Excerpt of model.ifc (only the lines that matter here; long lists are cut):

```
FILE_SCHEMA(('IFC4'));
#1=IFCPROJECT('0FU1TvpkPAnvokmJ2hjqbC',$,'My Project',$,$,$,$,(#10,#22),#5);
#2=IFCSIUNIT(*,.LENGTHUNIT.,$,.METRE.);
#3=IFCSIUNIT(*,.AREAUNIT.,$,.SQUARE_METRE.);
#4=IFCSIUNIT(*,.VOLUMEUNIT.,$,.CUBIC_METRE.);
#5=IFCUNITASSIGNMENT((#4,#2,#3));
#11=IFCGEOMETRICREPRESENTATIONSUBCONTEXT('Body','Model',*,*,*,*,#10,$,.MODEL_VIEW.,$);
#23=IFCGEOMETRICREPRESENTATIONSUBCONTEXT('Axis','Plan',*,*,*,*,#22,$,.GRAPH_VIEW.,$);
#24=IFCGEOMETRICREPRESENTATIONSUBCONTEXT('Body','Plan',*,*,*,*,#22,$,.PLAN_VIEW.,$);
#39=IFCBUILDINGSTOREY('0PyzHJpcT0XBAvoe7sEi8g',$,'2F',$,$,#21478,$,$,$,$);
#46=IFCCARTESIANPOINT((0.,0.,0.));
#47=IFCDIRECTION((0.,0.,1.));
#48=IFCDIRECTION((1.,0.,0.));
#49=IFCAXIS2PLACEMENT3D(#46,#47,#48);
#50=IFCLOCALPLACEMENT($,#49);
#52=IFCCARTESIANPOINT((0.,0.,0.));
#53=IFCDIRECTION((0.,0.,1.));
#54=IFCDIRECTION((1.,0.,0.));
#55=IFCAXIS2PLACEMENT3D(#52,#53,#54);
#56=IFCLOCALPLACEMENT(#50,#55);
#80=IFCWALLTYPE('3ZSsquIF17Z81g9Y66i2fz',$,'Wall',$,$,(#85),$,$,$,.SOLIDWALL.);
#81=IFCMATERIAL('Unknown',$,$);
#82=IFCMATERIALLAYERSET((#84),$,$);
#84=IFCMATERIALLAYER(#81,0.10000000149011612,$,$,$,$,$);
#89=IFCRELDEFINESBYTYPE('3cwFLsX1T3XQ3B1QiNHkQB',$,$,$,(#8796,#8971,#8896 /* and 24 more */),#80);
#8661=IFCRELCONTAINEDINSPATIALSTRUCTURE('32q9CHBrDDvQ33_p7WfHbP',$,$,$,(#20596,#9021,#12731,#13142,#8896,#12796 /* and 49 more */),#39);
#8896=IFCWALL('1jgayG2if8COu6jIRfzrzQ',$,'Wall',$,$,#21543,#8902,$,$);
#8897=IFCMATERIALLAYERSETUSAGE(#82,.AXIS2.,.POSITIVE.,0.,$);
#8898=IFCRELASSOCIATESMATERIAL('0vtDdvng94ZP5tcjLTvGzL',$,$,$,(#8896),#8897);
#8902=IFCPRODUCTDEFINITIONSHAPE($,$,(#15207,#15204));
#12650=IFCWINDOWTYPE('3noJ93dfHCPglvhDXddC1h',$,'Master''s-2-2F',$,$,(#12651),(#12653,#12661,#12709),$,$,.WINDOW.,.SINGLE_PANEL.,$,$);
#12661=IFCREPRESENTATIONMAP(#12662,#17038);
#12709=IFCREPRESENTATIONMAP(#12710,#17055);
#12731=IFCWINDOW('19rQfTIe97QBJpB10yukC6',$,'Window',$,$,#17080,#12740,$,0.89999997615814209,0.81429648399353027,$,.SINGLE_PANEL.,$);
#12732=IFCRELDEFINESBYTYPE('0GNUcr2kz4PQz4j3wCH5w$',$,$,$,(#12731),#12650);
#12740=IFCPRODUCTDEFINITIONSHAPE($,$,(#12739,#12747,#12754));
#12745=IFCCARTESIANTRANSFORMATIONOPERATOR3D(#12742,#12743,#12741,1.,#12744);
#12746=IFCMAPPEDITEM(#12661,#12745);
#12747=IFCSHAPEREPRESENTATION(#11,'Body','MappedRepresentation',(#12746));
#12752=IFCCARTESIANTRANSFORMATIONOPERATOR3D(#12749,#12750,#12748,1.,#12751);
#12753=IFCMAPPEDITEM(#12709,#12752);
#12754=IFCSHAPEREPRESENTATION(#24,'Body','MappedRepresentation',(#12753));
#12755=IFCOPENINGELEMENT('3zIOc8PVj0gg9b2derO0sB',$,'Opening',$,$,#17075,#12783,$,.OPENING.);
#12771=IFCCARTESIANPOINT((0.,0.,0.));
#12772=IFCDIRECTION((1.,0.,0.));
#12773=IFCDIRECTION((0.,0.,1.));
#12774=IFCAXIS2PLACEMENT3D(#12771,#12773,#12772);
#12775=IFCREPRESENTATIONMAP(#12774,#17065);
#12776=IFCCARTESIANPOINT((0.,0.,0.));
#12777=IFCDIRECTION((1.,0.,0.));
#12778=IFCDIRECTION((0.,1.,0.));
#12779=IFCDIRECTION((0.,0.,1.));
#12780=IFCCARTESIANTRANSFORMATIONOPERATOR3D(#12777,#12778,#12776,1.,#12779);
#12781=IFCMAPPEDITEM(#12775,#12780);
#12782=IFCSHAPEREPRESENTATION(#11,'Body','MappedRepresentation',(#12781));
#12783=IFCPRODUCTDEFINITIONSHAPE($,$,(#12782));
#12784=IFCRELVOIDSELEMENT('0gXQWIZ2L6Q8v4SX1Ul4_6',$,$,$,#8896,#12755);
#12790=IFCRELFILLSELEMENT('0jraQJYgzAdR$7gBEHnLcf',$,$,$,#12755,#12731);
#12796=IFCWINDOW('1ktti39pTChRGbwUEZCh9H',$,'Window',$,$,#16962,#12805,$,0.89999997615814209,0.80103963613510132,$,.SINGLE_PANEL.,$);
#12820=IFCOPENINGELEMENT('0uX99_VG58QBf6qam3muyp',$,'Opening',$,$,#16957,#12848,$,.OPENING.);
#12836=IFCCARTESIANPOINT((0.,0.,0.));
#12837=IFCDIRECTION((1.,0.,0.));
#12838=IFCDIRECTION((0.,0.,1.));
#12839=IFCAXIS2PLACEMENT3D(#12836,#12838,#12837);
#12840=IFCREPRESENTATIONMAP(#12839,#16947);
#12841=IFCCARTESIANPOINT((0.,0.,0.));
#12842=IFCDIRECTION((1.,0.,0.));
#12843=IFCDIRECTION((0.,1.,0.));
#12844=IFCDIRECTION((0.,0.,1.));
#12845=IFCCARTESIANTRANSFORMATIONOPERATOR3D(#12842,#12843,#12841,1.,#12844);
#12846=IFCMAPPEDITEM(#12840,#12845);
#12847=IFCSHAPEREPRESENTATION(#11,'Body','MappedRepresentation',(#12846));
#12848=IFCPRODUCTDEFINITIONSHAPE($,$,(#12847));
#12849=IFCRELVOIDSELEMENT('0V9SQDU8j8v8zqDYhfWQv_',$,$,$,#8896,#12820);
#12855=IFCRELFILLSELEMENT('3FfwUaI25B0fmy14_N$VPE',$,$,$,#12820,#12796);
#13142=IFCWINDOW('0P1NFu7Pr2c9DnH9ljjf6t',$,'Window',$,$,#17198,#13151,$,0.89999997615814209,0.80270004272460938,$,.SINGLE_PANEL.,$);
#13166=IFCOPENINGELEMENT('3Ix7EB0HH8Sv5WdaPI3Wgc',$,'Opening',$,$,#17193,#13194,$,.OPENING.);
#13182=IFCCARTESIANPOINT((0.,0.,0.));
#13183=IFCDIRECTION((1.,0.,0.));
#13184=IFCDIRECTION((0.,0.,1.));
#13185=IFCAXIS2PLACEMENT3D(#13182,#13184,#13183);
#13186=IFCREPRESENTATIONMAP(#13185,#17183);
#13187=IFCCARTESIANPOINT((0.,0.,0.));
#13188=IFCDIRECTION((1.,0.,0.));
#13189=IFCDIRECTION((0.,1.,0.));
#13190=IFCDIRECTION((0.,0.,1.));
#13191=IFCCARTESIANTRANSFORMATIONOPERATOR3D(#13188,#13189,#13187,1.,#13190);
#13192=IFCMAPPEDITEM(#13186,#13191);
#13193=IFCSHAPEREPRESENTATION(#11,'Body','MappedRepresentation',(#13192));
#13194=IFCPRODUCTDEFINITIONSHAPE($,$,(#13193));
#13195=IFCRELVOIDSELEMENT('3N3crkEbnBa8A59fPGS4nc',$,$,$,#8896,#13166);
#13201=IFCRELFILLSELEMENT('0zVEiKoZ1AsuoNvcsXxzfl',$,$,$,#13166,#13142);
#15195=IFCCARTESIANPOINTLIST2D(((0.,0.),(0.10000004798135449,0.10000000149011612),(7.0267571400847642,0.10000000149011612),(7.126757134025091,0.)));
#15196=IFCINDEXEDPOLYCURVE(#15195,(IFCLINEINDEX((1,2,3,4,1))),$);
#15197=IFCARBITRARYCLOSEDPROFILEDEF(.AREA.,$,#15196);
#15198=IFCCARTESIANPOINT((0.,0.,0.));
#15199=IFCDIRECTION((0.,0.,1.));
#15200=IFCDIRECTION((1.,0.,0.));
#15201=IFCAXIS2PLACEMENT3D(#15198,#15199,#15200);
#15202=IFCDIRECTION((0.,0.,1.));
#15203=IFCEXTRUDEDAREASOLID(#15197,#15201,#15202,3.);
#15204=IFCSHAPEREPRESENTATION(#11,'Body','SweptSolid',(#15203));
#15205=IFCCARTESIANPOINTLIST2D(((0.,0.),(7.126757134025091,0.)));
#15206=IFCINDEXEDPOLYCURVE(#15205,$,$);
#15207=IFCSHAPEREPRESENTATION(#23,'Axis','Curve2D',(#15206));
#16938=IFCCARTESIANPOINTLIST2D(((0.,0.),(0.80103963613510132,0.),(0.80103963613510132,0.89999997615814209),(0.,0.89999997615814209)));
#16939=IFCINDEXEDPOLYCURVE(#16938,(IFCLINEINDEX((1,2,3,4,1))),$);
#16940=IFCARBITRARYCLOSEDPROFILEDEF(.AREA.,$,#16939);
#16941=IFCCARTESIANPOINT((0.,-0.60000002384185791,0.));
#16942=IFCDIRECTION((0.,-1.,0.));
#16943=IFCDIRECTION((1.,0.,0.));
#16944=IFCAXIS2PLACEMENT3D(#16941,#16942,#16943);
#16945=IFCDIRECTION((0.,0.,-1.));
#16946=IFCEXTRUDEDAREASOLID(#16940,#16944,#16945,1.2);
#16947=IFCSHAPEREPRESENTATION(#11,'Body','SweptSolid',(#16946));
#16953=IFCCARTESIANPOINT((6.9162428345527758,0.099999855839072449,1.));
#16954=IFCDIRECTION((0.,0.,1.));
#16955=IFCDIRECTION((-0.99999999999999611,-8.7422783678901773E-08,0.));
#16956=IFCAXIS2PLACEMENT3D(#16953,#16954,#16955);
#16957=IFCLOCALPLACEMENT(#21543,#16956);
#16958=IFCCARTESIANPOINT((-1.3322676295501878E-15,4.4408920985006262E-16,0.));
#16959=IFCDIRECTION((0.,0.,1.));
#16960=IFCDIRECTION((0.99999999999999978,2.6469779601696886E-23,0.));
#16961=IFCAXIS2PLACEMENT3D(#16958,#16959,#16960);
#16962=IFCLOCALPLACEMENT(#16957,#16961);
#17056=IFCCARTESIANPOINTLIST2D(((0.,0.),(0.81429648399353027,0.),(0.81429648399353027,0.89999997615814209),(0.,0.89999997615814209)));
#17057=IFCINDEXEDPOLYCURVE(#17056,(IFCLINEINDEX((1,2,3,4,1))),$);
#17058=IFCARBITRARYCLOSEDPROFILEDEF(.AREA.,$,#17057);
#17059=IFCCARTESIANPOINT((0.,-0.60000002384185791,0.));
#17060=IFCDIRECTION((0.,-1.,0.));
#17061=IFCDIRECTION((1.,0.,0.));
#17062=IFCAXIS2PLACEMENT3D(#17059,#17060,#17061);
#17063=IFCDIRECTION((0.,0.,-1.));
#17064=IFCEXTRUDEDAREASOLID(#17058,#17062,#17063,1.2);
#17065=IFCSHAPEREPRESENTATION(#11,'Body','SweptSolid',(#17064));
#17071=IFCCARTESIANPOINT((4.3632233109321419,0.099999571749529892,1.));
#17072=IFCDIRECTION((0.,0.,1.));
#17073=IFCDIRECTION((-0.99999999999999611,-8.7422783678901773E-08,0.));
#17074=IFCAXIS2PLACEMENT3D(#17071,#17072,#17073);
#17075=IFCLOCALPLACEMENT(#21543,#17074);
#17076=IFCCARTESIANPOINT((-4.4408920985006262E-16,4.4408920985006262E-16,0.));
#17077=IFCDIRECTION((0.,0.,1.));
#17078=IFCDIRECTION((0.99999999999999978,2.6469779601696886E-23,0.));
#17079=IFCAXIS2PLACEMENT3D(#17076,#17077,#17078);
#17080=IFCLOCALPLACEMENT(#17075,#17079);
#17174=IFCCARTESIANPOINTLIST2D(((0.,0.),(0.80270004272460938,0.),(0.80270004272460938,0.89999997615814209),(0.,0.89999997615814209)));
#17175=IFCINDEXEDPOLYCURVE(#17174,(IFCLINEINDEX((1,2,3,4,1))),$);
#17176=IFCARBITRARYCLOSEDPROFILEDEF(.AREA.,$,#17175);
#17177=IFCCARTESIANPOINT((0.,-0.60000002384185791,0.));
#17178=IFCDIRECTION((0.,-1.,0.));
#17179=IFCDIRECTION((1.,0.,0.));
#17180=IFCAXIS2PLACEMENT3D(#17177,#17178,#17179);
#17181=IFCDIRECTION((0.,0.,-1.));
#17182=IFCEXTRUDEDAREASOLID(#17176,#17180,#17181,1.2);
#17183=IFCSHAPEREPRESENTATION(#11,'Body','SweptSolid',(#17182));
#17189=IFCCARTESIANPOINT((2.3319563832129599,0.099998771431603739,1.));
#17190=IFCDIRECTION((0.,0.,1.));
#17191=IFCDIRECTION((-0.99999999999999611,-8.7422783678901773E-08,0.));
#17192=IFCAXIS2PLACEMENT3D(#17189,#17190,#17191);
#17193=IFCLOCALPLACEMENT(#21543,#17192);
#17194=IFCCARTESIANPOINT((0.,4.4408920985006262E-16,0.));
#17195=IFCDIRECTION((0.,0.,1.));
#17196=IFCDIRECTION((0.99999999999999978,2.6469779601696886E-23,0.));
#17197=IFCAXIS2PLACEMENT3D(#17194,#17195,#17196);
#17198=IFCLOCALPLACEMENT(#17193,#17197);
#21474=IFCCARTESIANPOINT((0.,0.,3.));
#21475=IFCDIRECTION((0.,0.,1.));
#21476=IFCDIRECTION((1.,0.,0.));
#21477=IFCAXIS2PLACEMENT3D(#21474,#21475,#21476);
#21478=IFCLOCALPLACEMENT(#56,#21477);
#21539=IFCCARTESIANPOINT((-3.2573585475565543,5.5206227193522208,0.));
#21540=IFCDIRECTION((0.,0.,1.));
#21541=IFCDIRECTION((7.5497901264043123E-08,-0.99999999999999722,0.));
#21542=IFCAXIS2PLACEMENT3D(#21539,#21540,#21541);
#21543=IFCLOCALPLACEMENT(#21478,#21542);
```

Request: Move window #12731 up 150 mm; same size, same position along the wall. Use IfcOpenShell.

```python
import numpy as np
import ifcopenshell
import ifcopenshell.api.geometry
import ifcopenshell.util.placement
import ifcopenshell.util.unit

model = ifcopenshell.open("model.ifc")
unit_scale = ifcopenshell.util.unit.calculate_unit_scale(model)

window = model.by_guid("19rQfTIe97QBJpB10yukC6")
opening = window.FillsVoids[0].RelatingOpeningElement
dz = 0.15 / unit_scale

shift = np.array([0.0, 0.0, dz])
# The window is placed relative to its opening, so it follows when the opening moves.
matrix = ifcopenshell.util.placement.get_local_placement(opening.ObjectPlacement)
matrix[:3, 3] += shift
ifcopenshell.api.geometry.edit_object_placement(
    model, product=opening, matrix=matrix, is_si=False, should_transform_children=True
)

print(f"moved by {dz * unit_scale:+.3f} m")

model.write("model_updated.ifc")
```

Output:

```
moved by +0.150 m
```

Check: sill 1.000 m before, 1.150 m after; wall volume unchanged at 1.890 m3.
